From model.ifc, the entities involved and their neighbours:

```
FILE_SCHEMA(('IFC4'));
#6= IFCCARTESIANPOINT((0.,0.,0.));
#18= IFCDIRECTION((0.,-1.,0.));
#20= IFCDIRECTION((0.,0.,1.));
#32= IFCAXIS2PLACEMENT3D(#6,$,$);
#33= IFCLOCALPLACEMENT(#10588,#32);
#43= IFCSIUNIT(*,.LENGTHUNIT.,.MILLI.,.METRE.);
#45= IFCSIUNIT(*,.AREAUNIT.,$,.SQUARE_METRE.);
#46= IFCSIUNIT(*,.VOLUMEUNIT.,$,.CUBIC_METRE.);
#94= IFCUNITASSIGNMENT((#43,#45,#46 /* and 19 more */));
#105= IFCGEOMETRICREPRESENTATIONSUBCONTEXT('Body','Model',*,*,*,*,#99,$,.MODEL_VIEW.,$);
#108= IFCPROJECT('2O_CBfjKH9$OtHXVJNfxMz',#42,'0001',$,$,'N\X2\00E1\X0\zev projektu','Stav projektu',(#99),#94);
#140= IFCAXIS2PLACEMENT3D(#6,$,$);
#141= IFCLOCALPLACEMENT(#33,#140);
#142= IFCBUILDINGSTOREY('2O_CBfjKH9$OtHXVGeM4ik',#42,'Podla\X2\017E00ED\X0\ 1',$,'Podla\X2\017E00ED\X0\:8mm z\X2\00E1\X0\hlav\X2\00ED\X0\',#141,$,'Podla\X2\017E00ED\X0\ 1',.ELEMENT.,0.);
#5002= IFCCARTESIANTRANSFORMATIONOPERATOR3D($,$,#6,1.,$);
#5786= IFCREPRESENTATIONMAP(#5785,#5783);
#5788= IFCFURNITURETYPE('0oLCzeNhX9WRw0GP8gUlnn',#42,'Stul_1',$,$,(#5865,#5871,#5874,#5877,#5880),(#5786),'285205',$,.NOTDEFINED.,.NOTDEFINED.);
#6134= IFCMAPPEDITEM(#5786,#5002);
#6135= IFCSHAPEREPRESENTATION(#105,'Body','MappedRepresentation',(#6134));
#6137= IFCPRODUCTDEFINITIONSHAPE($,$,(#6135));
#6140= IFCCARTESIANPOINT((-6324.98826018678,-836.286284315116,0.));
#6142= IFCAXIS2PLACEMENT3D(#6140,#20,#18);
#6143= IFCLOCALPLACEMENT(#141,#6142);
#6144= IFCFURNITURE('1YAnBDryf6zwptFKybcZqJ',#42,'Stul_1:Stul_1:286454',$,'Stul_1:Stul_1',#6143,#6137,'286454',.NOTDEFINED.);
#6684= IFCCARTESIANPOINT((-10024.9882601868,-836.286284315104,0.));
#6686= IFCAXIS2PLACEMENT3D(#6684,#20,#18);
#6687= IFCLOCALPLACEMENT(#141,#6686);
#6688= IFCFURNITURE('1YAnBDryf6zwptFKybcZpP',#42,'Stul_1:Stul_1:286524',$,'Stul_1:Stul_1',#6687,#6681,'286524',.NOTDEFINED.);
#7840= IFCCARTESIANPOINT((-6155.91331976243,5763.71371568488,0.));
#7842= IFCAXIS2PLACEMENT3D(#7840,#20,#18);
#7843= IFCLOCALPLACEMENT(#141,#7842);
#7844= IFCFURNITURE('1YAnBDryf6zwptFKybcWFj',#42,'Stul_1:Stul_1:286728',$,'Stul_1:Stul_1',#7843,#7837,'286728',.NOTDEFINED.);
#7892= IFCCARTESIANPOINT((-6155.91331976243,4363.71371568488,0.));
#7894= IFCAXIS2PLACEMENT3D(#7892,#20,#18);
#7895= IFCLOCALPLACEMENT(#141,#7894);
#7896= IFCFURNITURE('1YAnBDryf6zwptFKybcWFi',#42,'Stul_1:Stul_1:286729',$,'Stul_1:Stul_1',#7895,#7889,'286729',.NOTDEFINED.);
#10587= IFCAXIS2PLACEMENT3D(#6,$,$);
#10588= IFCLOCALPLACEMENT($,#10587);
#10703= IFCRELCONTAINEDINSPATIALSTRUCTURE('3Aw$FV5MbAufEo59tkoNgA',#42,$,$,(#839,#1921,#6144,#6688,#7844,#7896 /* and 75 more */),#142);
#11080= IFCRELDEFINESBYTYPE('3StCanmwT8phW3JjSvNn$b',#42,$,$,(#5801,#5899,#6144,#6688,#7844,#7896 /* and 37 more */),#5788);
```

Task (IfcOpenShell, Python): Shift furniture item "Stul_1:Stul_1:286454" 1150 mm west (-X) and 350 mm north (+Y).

```python
import ifcopenshell
import ifcopenshell.api.geometry
import ifcopenshell.util.placement
import ifcopenshell.util.unit

model = ifcopenshell.open("model.ifc")
unit_scale = ifcopenshell.util.unit.calculate_unit_scale(model)

item = model.by_guid("1YAnBDryf6zwptFKybcZqJ")
matrix = ifcopenshell.util.placement.get_local_placement(item.ObjectPlacement)
matrix[0, 3] -= 1.15 / unit_scale
matrix[1, 3] += 0.35 / unit_scale
ifcopenshell.api.geometry.edit_object_placement(model, product=item, matrix=matrix, is_si=False)

print(ifcopenshell.util.placement.get_local_placement(item.ObjectPlacement).round(3) + 0.0)

model.write("model_edited.ifc")
```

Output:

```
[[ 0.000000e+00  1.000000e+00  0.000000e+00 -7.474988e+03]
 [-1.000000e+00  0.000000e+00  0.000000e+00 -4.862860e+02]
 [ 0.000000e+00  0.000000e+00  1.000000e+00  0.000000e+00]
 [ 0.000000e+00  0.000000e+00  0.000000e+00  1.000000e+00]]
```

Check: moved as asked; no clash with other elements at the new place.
